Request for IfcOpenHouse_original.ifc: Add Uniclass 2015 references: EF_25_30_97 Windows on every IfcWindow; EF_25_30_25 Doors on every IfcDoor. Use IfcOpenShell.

First a look at what the model holds.

```python
import ifcopenshell

model = ifcopenshell.open("IfcOpenHouse_original.ifc")
print(model.schema)
print("classifications:", [c.Name for c in model.by_type("IfcClassification")])
for ifc_class in ("IfcDoor", "IfcRoof", "IfcStair", "IfcWall", "IfcWindow"):
    print(ifc_class, len(model.by_type(ifc_class)))
```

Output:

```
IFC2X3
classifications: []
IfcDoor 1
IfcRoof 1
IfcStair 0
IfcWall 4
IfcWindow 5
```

```python
import ifcopenshell
import ifcopenshell.api.classification

model = ifcopenshell.open("IfcOpenHouse_original.ifc")

# IFC2X3 requires Source and Edition and has no link from the project to the system.
system = model.create_entity("IfcClassification", Source="NBS", Edition="2015", Name="Uniclass 2015")

codes = {
    "IfcWindow": ("EF_25_30_97", "Windows"),
    "IfcDoor": ("EF_25_30_25", "Doors"),
}
for ifc_class, (code, name) in codes.items():
    products = model.by_type(ifc_class)
    ifcopenshell.api.classification.add_reference(
        model, products=products, classification=system, identification=code, name=name
    )
    print(code, len(products))

model.write("IfcOpenHouse_original_v2.ifc")
```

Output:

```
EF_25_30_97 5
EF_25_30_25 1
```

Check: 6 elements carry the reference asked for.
